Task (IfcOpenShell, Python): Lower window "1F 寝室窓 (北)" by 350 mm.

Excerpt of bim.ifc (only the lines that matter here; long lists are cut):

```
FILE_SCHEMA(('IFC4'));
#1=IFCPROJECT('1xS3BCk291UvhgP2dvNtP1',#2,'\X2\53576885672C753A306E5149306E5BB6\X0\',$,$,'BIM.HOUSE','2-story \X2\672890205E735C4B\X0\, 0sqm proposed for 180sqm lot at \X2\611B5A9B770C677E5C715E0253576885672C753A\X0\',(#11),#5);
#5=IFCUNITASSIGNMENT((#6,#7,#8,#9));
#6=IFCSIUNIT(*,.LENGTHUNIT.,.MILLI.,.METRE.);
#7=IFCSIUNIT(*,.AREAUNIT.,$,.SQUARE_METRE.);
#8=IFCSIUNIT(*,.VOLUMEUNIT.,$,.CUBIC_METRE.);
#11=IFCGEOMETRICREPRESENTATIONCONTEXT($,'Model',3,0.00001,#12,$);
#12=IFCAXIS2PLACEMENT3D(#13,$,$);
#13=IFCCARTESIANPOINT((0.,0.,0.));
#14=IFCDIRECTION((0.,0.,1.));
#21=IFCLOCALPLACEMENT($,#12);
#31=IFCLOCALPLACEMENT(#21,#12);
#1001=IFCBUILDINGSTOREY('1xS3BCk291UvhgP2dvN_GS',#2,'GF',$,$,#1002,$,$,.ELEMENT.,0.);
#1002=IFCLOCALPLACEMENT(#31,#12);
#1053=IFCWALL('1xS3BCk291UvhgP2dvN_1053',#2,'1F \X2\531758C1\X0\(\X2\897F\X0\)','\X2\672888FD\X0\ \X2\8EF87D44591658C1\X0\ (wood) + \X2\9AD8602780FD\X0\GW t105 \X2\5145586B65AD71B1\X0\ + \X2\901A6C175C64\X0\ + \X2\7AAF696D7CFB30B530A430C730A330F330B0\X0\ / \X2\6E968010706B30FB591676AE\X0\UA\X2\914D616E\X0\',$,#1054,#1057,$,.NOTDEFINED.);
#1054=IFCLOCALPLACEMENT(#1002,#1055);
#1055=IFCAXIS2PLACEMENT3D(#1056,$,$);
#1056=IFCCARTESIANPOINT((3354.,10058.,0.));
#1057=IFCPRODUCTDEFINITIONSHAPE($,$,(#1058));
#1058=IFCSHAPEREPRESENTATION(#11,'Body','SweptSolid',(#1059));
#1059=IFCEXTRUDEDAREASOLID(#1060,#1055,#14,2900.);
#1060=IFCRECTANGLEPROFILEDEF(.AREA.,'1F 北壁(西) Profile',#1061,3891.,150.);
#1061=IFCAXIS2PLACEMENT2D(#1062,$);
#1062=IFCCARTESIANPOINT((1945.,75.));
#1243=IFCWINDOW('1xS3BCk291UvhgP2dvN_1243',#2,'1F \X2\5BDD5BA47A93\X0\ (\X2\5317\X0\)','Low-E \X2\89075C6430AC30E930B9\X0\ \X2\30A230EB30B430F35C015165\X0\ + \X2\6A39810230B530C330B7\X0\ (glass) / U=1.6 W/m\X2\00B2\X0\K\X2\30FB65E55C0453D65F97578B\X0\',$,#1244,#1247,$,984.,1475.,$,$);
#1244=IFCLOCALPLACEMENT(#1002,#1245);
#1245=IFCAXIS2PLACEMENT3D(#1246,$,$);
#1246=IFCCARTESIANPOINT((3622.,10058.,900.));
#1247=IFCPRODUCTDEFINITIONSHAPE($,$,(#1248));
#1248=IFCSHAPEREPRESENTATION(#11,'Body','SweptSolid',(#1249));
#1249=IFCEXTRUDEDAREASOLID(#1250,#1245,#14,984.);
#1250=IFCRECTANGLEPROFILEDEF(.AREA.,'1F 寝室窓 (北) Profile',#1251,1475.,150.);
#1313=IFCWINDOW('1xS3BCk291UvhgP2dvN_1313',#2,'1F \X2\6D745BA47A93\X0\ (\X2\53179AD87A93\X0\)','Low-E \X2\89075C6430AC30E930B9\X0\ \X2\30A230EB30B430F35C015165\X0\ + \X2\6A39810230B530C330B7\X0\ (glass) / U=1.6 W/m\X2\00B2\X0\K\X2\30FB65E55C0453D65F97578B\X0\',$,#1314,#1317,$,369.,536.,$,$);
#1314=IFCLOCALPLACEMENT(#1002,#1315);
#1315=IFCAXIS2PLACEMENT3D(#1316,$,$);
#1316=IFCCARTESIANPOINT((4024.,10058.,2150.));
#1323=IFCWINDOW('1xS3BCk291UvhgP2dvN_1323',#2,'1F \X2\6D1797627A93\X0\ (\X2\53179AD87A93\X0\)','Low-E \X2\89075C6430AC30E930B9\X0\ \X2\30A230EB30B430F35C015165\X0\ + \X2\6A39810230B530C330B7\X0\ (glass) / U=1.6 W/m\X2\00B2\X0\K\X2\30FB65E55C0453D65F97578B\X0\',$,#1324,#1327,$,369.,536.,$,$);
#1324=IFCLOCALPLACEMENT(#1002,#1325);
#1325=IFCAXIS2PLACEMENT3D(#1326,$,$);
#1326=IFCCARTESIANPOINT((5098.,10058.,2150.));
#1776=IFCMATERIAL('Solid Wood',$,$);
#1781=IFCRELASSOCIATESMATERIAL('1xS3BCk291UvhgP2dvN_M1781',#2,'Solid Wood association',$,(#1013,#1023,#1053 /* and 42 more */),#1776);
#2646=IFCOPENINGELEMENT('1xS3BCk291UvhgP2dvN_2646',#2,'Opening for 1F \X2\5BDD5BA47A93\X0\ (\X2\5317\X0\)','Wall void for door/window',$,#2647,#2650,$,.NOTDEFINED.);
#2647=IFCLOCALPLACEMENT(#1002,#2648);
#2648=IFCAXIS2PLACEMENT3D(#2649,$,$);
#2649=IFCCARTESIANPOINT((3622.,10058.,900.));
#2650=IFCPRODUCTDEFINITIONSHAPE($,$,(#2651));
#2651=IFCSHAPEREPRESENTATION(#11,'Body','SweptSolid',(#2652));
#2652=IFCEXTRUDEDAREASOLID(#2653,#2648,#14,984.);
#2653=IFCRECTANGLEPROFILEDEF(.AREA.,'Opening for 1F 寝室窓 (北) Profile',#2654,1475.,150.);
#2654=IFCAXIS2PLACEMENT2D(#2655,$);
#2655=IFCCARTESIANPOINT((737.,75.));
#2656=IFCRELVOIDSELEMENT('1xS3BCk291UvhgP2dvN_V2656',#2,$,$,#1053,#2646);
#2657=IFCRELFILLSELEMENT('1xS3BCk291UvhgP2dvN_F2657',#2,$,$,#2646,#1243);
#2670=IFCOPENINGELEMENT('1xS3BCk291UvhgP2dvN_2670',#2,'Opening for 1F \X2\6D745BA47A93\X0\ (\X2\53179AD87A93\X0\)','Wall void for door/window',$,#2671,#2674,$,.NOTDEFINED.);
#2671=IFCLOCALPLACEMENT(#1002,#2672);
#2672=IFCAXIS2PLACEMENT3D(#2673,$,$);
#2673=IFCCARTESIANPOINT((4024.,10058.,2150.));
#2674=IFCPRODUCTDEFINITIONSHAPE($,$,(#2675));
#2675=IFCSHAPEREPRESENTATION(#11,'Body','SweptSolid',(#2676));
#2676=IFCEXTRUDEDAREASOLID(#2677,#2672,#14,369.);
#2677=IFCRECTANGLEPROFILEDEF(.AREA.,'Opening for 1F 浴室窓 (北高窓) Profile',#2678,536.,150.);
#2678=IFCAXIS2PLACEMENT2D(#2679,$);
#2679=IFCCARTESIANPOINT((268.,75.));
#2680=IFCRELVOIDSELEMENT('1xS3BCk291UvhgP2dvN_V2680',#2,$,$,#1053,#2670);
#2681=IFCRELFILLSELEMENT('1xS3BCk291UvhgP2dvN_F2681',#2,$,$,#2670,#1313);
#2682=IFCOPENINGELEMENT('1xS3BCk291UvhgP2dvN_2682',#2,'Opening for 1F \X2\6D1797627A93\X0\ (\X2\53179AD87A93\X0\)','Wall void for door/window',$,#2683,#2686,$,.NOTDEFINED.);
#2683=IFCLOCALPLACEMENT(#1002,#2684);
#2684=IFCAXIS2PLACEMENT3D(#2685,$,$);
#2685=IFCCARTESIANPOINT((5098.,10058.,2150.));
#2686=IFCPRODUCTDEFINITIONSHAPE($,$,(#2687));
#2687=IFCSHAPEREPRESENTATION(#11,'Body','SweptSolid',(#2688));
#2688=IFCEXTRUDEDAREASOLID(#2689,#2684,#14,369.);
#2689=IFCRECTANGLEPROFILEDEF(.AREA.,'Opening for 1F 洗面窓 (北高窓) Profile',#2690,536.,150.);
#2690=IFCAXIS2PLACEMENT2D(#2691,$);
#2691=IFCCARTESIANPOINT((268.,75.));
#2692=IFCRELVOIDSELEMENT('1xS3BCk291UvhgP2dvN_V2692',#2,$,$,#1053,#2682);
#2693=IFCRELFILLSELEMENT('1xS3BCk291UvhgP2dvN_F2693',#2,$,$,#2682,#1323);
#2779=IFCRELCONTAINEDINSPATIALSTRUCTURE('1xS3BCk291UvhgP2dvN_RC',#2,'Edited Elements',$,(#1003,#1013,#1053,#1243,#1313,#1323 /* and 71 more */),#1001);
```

```python
import numpy as np
import ifcopenshell
import ifcopenshell.api.geometry
import ifcopenshell.util.placement
import ifcopenshell.util.unit

model = ifcopenshell.open("bim.ifc")
unit_scale = ifcopenshell.util.unit.calculate_unit_scale(model)

window = model.by_guid("1xS3BCk291UvhgP2dvN_1243")
opening = window.FillsVoids[0].RelatingOpeningElement
dz = -350.0

shift = np.array([0.0, 0.0, dz])
# The window is not placed relative to its opening, so move both.
for product in (opening, window):
    matrix = ifcopenshell.util.placement.get_local_placement(product.ObjectPlacement)
    matrix[:3, 3] += shift
    ifcopenshell.api.geometry.edit_object_placement(model, product=product, matrix=matrix, is_si=False)

print(f"moved by {dz * unit_scale:+.3f} m")

model.write("bim_v2.ifc")
```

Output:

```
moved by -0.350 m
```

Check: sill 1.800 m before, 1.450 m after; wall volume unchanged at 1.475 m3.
